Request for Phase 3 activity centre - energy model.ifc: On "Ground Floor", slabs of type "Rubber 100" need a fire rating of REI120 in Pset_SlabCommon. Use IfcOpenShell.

First a look at what the model holds.

```python
import ifcopenshell
import ifcopenshell.util.element

model = ifcopenshell.open("Phase 3 activity centre - energy model.ifc")
print(model.schema)
storey = next(s for s in model.by_type("IfcBuildingStorey") if s.Name == "Ground Floor")
slabs = [e for e in ifcopenshell.util.element.get_decomposition(storey) if e.is_a("IfcSlab")]
seen = {}
for e in slabs:
    element_type = ifcopenshell.util.element.get_type(e)
    key = (element_type.Name if element_type != e and element_type else None, ifcopenshell.util.element.get_pset(e, "Pset_SlabCommon", "FireRating"))
    seen[key] = seen.get(key, 0) + 1
for (name, value), count in sorted(seen.items(), key=str):
    print(count, "x", name, "|", value)
```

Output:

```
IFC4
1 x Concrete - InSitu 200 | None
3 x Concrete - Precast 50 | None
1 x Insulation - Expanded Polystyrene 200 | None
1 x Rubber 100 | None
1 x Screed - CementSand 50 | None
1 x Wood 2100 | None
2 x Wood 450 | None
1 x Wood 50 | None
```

```python
import ifcopenshell
import ifcopenshell.api.pset
import ifcopenshell.util.element

model = ifcopenshell.open("Phase 3 activity centre - energy model.ifc")

storey = next(s for s in model.by_type("IfcBuildingStorey") if s.Name == "Ground Floor")
slabs = [e for e in ifcopenshell.util.element.get_decomposition(storey) if e.is_a("IfcSlab")]

count = 0
for e in slabs:
    element_type = ifcopenshell.util.element.get_type(e)
    if element_type in (None, e) or element_type.Name != "Rubber 100":
        continue
    # add_pset returns the element's existing set when there is one.
    pset = ifcopenshell.api.pset.add_pset(model, product=e, name="Pset_SlabCommon")
    ifcopenshell.api.pset.edit_pset(model, pset=pset, properties={"FireRating": "REI120"})
    count += 1

print(count, "slabs updated")

model.write("Phase 3 activity centre - energy model-out.ifc")
```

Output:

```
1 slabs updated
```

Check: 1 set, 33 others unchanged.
